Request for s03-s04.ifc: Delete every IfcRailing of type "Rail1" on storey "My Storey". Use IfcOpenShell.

First a look at what the model holds.

```python
import ifcopenshell
import ifcopenshell.util.element

model = ifcopenshell.open("s03-s04.ifc")
print(model.schema)
storey = next(s for s in model.by_type("IfcBuildingStorey") if s.Name == "My Storey")
railings = [e for e in ifcopenshell.util.element.get_decomposition(storey) if e.is_a("IfcRailing")]
seen = {}
for e in railings:
    element_type = ifcopenshell.util.element.get_type(e)
    name = element_type.Name if element_type not in (None, e) else None
    seen[name] = seen.get(name, 0) + 1
for name, count in sorted(seen.items(), key=str):
    print(count, "x", name)
```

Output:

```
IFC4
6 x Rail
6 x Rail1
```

```python
import ifcopenshell
import ifcopenshell.api.root
import ifcopenshell.util.element

model = ifcopenshell.open("s03-s04.ifc")

storey = next(s for s in model.by_type("IfcBuildingStorey") if s.Name == "My Storey")
railings = [e for e in ifcopenshell.util.element.get_decomposition(storey) if e.is_a("IfcRailing")]
targets = [e for e in railings if (t := ifcopenshell.util.element.get_type(e)) not in (None, e) and t.Name == "Rail1"]

for e in targets:
    ifcopenshell.api.root.remove_product(model, product=e)
print(len(targets), "removed")

model.write("s03-s04_rev.ifc")
```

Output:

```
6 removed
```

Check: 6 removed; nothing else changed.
